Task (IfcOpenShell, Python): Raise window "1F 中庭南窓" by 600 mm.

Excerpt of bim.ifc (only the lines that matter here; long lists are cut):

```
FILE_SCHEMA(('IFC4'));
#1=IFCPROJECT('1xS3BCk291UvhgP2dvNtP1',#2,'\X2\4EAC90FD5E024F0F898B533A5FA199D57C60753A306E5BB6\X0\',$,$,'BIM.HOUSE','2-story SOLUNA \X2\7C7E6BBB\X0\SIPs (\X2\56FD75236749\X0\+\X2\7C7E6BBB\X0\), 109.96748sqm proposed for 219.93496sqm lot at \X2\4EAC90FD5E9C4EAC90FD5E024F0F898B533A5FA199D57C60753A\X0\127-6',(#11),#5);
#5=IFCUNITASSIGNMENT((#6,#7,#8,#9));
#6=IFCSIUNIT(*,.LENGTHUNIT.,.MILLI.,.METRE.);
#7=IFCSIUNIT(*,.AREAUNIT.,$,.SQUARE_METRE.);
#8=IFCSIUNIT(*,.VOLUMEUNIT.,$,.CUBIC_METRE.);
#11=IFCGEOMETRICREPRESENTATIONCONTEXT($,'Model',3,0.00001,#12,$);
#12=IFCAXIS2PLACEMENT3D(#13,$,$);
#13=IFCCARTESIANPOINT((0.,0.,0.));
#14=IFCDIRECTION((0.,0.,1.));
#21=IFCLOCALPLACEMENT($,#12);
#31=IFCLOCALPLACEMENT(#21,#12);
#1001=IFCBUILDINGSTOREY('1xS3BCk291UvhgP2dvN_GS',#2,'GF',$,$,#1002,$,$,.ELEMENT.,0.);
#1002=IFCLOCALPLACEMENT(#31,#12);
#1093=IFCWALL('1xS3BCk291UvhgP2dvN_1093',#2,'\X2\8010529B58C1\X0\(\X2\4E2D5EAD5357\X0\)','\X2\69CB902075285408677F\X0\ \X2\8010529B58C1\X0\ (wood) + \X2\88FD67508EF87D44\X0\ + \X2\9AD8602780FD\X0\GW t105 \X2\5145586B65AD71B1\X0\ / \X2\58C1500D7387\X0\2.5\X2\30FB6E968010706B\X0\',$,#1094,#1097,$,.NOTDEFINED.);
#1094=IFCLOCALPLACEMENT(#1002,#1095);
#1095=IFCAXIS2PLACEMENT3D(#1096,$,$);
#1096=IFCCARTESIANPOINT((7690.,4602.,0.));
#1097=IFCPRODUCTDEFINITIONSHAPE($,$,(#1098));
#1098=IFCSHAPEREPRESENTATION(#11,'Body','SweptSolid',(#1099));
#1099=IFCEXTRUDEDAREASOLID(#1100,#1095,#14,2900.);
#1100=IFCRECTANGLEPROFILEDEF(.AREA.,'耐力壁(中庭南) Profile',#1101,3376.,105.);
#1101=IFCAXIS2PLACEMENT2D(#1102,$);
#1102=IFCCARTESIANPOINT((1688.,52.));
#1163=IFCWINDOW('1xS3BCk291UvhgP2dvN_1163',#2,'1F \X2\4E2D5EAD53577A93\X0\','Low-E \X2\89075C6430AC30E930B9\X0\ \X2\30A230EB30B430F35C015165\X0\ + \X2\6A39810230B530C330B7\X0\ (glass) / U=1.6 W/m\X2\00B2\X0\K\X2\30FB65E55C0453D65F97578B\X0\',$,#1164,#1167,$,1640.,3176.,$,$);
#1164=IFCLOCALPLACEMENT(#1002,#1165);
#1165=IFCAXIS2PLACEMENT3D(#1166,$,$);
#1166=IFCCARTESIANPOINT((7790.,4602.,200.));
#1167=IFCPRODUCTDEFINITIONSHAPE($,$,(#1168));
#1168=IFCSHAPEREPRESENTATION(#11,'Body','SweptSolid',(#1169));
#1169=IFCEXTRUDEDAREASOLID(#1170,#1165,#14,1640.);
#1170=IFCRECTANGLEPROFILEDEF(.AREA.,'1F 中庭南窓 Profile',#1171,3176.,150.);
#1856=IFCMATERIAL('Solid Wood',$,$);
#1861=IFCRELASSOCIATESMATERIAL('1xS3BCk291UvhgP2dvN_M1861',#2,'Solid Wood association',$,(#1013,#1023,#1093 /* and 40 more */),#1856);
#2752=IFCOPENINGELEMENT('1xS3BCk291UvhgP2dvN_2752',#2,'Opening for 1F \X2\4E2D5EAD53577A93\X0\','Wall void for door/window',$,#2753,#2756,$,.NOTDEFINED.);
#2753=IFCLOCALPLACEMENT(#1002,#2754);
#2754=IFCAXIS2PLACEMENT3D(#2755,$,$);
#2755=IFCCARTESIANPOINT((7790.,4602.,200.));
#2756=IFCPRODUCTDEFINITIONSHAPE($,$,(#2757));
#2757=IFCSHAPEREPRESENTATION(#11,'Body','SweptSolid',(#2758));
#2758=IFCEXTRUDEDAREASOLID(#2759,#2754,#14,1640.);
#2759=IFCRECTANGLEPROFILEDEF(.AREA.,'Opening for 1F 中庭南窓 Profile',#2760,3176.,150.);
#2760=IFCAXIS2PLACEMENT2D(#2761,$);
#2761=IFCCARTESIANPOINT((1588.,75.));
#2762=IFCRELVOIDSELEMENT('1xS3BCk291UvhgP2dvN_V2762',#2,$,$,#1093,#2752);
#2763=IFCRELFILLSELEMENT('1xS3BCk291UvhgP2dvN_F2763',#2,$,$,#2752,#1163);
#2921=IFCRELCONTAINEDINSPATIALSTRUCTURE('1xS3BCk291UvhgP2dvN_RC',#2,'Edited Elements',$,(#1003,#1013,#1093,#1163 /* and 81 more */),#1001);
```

```python
import numpy as np
import ifcopenshell
import ifcopenshell.api.geometry
import ifcopenshell.util.placement
import ifcopenshell.util.unit

model = ifcopenshell.open("bim.ifc")
unit_scale = ifcopenshell.util.unit.calculate_unit_scale(model)

window = model.by_guid("1xS3BCk291UvhgP2dvN_1163")
opening = window.FillsVoids[0].RelatingOpeningElement
dz = 0.6 / unit_scale

shift = np.array([0.0, 0.0, dz])
# The window is not placed relative to its opening, so move both.
for product in (opening, window):
    matrix = ifcopenshell.util.placement.get_local_placement(product.ObjectPlacement)
    matrix[:3, 3] += shift
    ifcopenshell.api.geometry.edit_object_placement(model, product=product, matrix=matrix, is_si=False)

print(f"moved by {dz * unit_scale:+.3f} m")

model.write("bim_updated.ifc")
```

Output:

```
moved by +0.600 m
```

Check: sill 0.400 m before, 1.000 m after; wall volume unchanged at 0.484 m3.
